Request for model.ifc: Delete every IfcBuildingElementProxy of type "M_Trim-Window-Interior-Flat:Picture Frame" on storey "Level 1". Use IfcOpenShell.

First a look at what the model holds.

```python
import ifcopenshell
import ifcopenshell.util.element

model = ifcopenshell.open("model.ifc")
print(model.schema)
storey = next(s for s in model.by_type("IfcBuildingStorey") if s.Name == "Level 1")
proxies = [e for e in ifcopenshell.util.element.get_decomposition(storey) if e.is_a("IfcBuildingElementProxy")]
seen = {}
for e in proxies:
    element_type = ifcopenshell.util.element.get_type(e)
    name = element_type.Name if element_type not in (None, e) else None
    seen[name] = seen.get(name, 0) + 1
for name, count in sorted(seen.items(), key=str):
    print(count, "x", name)
```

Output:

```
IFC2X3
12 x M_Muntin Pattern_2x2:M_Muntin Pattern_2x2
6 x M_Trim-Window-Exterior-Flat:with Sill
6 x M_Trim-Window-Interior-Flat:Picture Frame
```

```python
import ifcopenshell
import ifcopenshell.api.root
import ifcopenshell.util.element

model = ifcopenshell.open("model.ifc")

storey = next(s for s in model.by_type("IfcBuildingStorey") if s.Name == "Level 1")
proxies = [e for e in ifcopenshell.util.element.get_decomposition(storey) if e.is_a("IfcBuildingElementProxy")]
targets = [e for e in proxies if (t := ifcopenshell.util.element.get_type(e)) not in (None, e) and t.Name == "M_Trim-Window-Interior-Flat:Picture Frame"]

for e in targets:
    ifcopenshell.api.root.remove_product(model, product=e)
print(len(targets), "removed")

model.write("model_rev.ifc")
```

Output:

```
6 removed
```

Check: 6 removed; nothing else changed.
